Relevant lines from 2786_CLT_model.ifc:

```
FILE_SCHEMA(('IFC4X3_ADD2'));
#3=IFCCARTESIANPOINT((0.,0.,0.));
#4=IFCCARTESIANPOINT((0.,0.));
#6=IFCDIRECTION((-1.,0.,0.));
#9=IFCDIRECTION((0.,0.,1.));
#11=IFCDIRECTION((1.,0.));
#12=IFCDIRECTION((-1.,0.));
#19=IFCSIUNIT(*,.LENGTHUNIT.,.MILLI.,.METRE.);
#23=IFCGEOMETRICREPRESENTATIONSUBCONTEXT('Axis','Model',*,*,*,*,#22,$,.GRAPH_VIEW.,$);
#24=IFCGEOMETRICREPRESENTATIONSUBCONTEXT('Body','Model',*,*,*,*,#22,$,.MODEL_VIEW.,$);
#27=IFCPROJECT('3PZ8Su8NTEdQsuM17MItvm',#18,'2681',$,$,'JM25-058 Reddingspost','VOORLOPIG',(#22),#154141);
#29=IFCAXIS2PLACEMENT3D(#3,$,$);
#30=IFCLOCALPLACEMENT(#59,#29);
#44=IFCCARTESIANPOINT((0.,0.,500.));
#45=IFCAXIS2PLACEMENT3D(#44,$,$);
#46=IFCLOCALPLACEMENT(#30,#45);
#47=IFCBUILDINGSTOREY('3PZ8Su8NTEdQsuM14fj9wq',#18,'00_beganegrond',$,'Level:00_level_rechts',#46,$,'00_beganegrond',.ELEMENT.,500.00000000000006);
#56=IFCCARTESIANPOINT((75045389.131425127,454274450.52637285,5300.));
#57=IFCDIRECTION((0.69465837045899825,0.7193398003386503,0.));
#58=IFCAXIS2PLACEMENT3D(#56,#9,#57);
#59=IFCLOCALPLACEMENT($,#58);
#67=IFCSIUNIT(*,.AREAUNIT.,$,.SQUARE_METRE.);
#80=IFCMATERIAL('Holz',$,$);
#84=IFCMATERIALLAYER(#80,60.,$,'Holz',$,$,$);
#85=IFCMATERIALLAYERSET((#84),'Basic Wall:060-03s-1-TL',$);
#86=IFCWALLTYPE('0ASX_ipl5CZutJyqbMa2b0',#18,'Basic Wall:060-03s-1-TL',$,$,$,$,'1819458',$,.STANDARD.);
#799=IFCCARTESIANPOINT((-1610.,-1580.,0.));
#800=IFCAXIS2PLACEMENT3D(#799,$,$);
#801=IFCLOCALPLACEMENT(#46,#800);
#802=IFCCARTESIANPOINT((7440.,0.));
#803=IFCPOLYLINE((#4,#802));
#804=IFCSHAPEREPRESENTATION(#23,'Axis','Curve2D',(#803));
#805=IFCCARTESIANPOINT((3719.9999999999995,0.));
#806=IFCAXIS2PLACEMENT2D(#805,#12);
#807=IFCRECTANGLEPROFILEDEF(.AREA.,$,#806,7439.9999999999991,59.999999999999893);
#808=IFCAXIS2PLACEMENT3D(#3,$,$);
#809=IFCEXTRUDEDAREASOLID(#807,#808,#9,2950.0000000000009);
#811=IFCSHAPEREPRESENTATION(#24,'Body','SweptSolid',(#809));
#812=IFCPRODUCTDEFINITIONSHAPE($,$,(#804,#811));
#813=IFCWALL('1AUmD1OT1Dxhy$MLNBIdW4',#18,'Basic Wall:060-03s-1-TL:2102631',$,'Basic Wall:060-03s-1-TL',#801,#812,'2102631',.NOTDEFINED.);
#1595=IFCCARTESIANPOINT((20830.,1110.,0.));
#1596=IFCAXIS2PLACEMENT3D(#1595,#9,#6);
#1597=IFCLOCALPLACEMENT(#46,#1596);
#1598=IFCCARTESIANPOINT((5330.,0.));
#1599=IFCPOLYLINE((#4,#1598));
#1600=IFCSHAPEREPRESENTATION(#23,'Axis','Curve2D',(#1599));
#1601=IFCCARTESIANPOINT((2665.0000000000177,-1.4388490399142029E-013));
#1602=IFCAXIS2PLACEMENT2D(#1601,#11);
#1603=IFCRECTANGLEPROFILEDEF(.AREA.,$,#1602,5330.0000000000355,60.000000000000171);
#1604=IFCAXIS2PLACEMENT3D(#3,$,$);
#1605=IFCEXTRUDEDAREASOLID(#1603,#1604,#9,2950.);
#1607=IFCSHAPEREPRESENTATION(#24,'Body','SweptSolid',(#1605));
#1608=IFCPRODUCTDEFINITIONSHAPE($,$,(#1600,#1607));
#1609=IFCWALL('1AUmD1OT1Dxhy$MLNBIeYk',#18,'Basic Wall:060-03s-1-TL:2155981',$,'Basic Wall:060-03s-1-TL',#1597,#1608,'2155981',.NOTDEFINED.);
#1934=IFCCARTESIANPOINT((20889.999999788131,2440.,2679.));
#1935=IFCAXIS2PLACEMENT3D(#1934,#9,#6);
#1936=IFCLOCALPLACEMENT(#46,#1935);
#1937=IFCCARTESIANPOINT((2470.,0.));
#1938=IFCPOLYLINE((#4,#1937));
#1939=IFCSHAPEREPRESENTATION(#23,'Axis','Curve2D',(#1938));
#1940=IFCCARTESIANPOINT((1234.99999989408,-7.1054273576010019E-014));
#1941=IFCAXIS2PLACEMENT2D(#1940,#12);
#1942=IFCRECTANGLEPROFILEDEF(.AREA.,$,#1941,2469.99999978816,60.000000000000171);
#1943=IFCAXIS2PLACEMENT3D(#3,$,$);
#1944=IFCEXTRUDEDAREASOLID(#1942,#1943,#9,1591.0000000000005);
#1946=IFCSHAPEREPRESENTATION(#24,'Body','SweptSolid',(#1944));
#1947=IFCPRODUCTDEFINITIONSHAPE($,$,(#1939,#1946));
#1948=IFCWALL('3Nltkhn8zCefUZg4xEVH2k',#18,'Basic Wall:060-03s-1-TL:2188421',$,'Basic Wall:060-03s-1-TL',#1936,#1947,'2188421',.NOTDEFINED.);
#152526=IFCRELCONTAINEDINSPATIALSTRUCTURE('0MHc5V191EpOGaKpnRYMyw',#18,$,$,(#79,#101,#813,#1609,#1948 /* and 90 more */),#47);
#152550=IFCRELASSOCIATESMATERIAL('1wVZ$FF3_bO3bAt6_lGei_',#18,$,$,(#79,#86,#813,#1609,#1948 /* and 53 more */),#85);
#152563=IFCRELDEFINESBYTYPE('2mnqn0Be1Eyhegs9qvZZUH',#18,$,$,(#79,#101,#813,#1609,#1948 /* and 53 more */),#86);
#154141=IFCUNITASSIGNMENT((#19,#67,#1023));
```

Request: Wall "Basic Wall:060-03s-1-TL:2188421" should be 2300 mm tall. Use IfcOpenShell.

```python
import ifcopenshell
import ifcopenshell.geom
import ifcopenshell.util.representation
import ifcopenshell.util.shape

model = ifcopenshell.open("2786_CLT_model.ifc")
settings = ifcopenshell.geom.settings()


def volume(element):
    """Net volume in cubic metres, openings subtracted."""
    shape = ifcopenshell.geom.create_shape(settings, element)
    return ifcopenshell.util.shape.get_volume(shape.geometry)


wall = model.by_guid("3Nltkhn8zCefUZg4xEVH2k")
before = volume(wall)

body = ifcopenshell.util.representation.get_representation(wall, "Model", "Body")
solid = body.Items[0]
old_height = solid.Depth
solid.Depth = 2300.0
after = volume(wall)

print(f"height {old_height:g} -> {solid.Depth:g}, volume {before:.3f} -> {after:.3f} m3")

model.write("2786_CLT_model_v2.ifc")
```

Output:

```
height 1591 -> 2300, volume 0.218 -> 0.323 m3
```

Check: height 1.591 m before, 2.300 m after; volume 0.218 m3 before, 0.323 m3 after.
